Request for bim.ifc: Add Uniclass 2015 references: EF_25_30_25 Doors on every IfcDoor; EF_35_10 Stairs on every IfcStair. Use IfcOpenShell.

First a look at what the model holds.

```python
import ifcopenshell

model = ifcopenshell.open("bim.ifc")
print(model.schema)
print("classifications:", [c.Name for c in model.by_type("IfcClassification")])
for ifc_class in ("IfcDoor", "IfcRoof", "IfcStair", "IfcWall", "IfcWindow"):
    print(ifc_class, len(model.by_type(ifc_class)))
```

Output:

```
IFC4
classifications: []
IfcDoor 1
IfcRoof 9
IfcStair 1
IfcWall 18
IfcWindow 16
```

```python
import ifcopenshell
import ifcopenshell.api.classification

model = ifcopenshell.open("bim.ifc")

system = ifcopenshell.api.classification.add_classification(model, classification="Uniclass 2015")

codes = {
    "IfcDoor": ("EF_25_30_25", "Doors"),
    "IfcStair": ("EF_35_10", "Stairs"),
}
for ifc_class, (code, name) in codes.items():
    products = model.by_type(ifc_class)
    ifcopenshell.api.classification.add_reference(
        model, products=products, classification=system, identification=code, name=name
    )
    print(code, len(products))

model.write("bim_updated.ifc")
```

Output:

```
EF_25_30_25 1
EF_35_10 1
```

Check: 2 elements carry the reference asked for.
